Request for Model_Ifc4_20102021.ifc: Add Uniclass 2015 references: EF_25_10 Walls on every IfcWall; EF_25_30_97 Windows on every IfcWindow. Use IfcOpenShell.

First a look at what the model holds.

```python
import ifcopenshell

model = ifcopenshell.open("Model_Ifc4_20102021.ifc")
print(model.schema)
print("classifications:", [c.Name for c in model.by_type("IfcClassification")])
for ifc_class in ("IfcDoor", "IfcRoof", "IfcStair", "IfcWall", "IfcWindow"):
    print(ifc_class, len(model.by_type(ifc_class)))
```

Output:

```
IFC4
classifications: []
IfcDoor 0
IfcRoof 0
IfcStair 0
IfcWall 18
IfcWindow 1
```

```python
import ifcopenshell
import ifcopenshell.api.classification

model = ifcopenshell.open("Model_Ifc4_20102021.ifc")

system = ifcopenshell.api.classification.add_classification(model, classification="Uniclass 2015")

codes = {
    "IfcWall": ("EF_25_10", "Walls"),
    "IfcWindow": ("EF_25_30_97", "Windows"),
}
for ifc_class, (code, name) in codes.items():
    products = model.by_type(ifc_class)
    ifcopenshell.api.classification.add_reference(
        model, products=products, classification=system, identification=code, name=name
    )
    print(code, len(products))

model.write("Model_Ifc4_20102021_edited.ifc")
```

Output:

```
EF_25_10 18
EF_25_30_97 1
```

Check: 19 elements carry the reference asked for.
